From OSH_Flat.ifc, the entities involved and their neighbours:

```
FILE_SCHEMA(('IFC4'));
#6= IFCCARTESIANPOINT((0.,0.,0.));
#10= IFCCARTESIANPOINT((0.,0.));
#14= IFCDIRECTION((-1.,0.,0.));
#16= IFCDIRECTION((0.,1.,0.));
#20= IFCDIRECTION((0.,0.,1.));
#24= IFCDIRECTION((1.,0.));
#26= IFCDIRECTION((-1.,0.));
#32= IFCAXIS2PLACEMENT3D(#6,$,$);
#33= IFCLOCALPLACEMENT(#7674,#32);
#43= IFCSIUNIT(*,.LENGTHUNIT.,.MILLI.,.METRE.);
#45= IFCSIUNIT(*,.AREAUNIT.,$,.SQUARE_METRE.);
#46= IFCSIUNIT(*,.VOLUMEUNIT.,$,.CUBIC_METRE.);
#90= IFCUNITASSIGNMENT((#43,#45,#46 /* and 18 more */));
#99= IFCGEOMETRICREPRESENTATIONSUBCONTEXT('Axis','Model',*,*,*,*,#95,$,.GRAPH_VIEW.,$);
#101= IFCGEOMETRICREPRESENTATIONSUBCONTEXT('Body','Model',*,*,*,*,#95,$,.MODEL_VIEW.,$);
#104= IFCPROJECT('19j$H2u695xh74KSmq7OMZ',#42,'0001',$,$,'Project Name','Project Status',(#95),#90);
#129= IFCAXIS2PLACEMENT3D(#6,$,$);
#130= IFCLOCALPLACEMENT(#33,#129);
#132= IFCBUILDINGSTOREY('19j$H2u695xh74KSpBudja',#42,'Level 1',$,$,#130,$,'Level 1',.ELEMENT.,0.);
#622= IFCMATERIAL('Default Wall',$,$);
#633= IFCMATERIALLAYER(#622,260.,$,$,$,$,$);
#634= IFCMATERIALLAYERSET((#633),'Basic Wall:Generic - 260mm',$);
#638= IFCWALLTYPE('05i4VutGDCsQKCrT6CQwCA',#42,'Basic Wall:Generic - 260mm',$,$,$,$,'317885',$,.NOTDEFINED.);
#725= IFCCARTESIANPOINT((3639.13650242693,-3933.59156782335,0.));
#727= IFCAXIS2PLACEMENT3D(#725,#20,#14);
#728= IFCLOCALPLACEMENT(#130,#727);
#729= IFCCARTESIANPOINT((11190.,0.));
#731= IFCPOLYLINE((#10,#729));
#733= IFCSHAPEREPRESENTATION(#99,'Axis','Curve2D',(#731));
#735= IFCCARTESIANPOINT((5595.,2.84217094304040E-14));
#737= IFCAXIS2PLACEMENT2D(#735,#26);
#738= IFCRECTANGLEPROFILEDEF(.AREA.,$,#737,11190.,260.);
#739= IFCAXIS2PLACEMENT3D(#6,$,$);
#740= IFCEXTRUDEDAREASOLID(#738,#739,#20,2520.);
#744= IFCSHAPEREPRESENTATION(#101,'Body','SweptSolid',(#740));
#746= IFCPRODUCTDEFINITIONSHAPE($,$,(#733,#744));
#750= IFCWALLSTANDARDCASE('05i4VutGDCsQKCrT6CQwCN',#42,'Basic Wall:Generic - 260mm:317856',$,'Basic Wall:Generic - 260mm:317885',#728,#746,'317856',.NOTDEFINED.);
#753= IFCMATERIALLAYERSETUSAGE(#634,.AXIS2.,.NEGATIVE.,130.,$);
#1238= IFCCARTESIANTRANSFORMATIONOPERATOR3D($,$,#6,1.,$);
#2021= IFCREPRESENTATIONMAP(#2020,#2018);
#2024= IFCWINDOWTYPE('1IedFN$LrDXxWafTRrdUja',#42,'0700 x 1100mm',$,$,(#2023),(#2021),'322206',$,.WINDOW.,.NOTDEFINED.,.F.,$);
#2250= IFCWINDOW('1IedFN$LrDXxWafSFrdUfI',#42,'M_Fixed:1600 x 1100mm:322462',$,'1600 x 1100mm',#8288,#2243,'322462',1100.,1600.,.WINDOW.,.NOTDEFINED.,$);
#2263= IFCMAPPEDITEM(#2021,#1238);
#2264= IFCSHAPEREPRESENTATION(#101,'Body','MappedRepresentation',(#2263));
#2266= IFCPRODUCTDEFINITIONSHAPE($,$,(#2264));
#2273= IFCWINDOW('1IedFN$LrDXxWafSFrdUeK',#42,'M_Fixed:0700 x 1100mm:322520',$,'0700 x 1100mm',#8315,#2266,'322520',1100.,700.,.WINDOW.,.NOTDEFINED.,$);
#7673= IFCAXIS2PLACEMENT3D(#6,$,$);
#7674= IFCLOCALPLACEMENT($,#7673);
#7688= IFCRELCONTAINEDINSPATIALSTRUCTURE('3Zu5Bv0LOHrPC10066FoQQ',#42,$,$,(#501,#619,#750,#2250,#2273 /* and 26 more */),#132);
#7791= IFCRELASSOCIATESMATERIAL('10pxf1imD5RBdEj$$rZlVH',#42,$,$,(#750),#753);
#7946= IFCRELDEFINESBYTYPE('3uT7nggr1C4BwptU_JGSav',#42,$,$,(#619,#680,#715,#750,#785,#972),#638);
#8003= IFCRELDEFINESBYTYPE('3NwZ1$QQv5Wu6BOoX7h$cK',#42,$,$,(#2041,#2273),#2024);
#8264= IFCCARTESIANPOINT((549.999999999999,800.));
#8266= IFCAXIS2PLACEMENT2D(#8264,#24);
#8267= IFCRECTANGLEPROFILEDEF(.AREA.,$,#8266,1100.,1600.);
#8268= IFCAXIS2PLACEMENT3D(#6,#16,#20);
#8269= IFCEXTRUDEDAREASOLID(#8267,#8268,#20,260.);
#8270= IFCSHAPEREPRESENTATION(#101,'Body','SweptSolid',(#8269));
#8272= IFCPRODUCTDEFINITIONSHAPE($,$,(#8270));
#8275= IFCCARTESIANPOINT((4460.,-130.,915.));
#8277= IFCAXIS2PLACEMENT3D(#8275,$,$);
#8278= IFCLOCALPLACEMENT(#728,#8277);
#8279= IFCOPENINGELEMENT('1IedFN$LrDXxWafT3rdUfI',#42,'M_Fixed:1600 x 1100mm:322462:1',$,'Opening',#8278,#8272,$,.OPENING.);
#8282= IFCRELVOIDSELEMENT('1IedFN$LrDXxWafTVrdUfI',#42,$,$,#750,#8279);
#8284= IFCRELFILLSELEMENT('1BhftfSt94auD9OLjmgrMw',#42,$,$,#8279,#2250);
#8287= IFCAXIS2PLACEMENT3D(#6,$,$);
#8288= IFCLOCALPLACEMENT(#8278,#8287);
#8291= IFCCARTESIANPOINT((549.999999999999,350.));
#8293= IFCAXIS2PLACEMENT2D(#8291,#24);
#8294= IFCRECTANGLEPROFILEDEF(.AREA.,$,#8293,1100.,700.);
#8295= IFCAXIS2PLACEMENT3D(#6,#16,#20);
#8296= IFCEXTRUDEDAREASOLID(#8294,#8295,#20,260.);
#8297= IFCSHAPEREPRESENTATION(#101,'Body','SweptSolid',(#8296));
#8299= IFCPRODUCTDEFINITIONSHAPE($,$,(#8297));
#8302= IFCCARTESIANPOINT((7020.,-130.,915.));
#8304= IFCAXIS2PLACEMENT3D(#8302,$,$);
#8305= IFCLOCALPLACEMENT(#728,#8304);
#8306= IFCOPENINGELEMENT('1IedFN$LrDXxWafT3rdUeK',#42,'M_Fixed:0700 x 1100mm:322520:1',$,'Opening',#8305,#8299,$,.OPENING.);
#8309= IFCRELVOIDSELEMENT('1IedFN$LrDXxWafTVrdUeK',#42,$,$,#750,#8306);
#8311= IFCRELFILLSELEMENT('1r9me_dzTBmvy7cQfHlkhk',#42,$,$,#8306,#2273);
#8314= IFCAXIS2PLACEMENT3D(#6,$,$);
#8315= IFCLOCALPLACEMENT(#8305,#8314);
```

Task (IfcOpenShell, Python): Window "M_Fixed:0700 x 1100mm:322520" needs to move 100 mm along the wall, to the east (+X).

```python
import ifcopenshell
import ifcopenshell.api.geometry
import ifcopenshell.util.placement
import ifcopenshell.util.unit

model = ifcopenshell.open("OSH_Flat.ifc")
unit_scale = ifcopenshell.util.unit.calculate_unit_scale(model)

window = model.by_id(2273)
opening = window.FillsVoids[0].RelatingOpeningElement
wall = opening.VoidsElements[0].RelatingBuildingElement

wall_matrix = ifcopenshell.util.placement.get_local_placement(wall.ObjectPlacement)
shift = wall_matrix[:3, 0] * -0.1 / unit_scale
before = ifcopenshell.util.placement.get_local_placement(window.ObjectPlacement)[:3, 3].copy()

# The window is placed relative to its opening, so it follows when the opening moves.
matrix = ifcopenshell.util.placement.get_local_placement(opening.ObjectPlacement)
matrix[:3, 3] += shift
ifcopenshell.api.geometry.edit_object_placement(
    model, product=opening, matrix=matrix, is_si=False, should_transform_children=True
)

after = ifcopenshell.util.placement.get_local_placement(window.ObjectPlacement)[:3, 3]
print("window moved by", (after - before).round(3) + 0.0)

model.write("OSH_Flat_rev.ifc")
```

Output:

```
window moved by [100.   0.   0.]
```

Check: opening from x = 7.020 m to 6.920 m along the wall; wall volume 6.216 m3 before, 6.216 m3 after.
